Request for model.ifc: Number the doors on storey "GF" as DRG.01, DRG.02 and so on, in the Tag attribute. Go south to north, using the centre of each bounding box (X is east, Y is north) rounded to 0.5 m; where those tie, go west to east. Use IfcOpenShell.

First a look at what the model holds.

```python
import ifcopenshell
import ifcopenshell.util.element
import ifcopenshell.util.placement

model = ifcopenshell.open("model.ifc")
print(model.schema)
storey = next(s for s in model.by_type("IfcBuildingStorey") if s.Name == "GF")
doors = [e for e in ifcopenshell.util.element.get_decomposition(storey) if e.is_a("IfcDoor")]
for e in sorted(doors, key=lambda e: e.id()):
    origin = ifcopenshell.util.placement.get_local_placement(e.ObjectPlacement)[:3, 3]
    print(e.id(), e.Tag, e.Name, origin.round(2) + 0.0, sep=" | ")
```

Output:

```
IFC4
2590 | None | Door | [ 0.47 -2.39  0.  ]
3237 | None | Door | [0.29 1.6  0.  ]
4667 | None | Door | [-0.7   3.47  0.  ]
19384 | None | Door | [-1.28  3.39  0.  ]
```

```python
import ifcopenshell
import ifcopenshell.geom
import ifcopenshell.util.element
import ifcopenshell.util.shape

model = ifcopenshell.open("model.ifc")
settings = ifcopenshell.geom.settings()
settings.set("use-world-coords", True)


def centre(element):
    shape = ifcopenshell.geom.create_shape(settings, element)
    return ifcopenshell.util.shape.get_bbox_centroid(shape.geometry)


storey = next(s for s in model.by_type("IfcBuildingStorey") if s.Name == "GF")
doors = [e for e in ifcopenshell.util.element.get_decomposition(storey) if e.is_a("IfcDoor")]

# Insertion points can sit at a corner or the storey origin, so sort by the geometry (in metres).
centres = {e: centre(e) for e in doors}
doors.sort(key=lambda e: (round(centres[e][1] / 0.5), centres[e][0]))

for i, e in enumerate(doors, start=1):
    number = f"DRG.{i:02d}"
    e.Tag = number
    print(e.id(), number)

model.write("model_v2.ifc")
```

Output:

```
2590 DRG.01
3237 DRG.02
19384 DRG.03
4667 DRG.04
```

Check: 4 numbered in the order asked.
